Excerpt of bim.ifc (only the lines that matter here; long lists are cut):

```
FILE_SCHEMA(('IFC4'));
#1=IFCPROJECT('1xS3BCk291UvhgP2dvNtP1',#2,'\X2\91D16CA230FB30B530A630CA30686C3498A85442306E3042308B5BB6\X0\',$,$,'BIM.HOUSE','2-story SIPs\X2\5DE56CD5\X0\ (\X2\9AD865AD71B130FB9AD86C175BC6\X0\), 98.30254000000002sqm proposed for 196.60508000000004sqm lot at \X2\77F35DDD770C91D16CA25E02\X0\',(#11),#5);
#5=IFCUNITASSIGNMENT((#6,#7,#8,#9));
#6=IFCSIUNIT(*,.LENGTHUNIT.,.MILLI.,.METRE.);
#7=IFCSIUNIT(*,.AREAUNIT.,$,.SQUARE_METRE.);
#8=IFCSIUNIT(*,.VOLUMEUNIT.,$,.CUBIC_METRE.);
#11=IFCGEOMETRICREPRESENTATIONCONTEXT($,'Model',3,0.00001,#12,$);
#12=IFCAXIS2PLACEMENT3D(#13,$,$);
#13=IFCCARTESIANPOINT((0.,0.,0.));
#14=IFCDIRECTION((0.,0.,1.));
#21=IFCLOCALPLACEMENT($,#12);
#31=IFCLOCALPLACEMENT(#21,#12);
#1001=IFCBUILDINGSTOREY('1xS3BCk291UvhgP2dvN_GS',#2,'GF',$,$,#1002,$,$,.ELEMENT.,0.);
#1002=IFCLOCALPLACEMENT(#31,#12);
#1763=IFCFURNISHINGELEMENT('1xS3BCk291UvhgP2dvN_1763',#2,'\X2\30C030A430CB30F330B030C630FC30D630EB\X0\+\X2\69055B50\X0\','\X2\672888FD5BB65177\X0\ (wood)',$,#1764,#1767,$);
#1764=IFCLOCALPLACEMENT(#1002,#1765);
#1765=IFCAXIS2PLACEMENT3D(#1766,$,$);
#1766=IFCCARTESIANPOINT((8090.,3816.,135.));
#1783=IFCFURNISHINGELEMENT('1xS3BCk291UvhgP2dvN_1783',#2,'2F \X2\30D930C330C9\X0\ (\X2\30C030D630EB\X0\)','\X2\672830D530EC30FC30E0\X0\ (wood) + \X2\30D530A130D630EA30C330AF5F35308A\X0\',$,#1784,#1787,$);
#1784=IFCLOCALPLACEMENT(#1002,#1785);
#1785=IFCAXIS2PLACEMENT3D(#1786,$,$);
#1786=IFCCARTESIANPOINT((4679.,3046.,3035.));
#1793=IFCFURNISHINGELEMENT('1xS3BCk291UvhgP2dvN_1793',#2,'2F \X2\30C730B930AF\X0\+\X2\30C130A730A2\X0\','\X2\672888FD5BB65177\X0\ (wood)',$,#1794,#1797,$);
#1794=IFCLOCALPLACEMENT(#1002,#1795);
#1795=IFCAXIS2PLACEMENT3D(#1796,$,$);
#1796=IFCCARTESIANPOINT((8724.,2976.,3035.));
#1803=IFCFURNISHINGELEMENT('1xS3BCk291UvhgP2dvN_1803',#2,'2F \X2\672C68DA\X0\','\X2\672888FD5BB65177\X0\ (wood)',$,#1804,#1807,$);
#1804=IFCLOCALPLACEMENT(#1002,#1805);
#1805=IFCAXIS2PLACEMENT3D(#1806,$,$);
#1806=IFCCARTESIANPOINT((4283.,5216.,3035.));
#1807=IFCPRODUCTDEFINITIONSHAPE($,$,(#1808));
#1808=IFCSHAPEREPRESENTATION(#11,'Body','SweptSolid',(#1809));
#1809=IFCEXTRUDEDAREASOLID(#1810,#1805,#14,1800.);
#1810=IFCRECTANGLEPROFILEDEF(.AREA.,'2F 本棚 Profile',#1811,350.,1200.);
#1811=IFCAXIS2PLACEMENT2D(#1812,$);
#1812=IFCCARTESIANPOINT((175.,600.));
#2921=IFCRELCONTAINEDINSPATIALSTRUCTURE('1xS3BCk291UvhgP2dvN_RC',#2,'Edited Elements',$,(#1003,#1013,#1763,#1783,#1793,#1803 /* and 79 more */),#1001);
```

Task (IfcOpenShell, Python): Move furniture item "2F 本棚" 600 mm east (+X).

```python
import ifcopenshell
import ifcopenshell.api.geometry
import ifcopenshell.util.placement
import ifcopenshell.util.unit

model = ifcopenshell.open("bim.ifc")
unit_scale = ifcopenshell.util.unit.calculate_unit_scale(model)

item = model.by_guid("1xS3BCk291UvhgP2dvN_1803")
matrix = ifcopenshell.util.placement.get_local_placement(item.ObjectPlacement)
matrix[0, 3] += 0.6 / unit_scale
ifcopenshell.api.geometry.edit_object_placement(model, product=item, matrix=matrix, is_si=False)

print(ifcopenshell.util.placement.get_local_placement(item.ObjectPlacement).round(3) + 0.0)

model.write("bim_edited.ifc")
```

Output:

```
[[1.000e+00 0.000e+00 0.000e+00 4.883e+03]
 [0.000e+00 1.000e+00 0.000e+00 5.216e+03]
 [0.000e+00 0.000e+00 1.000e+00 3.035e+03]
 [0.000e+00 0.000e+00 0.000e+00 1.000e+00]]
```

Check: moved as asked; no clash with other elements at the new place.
